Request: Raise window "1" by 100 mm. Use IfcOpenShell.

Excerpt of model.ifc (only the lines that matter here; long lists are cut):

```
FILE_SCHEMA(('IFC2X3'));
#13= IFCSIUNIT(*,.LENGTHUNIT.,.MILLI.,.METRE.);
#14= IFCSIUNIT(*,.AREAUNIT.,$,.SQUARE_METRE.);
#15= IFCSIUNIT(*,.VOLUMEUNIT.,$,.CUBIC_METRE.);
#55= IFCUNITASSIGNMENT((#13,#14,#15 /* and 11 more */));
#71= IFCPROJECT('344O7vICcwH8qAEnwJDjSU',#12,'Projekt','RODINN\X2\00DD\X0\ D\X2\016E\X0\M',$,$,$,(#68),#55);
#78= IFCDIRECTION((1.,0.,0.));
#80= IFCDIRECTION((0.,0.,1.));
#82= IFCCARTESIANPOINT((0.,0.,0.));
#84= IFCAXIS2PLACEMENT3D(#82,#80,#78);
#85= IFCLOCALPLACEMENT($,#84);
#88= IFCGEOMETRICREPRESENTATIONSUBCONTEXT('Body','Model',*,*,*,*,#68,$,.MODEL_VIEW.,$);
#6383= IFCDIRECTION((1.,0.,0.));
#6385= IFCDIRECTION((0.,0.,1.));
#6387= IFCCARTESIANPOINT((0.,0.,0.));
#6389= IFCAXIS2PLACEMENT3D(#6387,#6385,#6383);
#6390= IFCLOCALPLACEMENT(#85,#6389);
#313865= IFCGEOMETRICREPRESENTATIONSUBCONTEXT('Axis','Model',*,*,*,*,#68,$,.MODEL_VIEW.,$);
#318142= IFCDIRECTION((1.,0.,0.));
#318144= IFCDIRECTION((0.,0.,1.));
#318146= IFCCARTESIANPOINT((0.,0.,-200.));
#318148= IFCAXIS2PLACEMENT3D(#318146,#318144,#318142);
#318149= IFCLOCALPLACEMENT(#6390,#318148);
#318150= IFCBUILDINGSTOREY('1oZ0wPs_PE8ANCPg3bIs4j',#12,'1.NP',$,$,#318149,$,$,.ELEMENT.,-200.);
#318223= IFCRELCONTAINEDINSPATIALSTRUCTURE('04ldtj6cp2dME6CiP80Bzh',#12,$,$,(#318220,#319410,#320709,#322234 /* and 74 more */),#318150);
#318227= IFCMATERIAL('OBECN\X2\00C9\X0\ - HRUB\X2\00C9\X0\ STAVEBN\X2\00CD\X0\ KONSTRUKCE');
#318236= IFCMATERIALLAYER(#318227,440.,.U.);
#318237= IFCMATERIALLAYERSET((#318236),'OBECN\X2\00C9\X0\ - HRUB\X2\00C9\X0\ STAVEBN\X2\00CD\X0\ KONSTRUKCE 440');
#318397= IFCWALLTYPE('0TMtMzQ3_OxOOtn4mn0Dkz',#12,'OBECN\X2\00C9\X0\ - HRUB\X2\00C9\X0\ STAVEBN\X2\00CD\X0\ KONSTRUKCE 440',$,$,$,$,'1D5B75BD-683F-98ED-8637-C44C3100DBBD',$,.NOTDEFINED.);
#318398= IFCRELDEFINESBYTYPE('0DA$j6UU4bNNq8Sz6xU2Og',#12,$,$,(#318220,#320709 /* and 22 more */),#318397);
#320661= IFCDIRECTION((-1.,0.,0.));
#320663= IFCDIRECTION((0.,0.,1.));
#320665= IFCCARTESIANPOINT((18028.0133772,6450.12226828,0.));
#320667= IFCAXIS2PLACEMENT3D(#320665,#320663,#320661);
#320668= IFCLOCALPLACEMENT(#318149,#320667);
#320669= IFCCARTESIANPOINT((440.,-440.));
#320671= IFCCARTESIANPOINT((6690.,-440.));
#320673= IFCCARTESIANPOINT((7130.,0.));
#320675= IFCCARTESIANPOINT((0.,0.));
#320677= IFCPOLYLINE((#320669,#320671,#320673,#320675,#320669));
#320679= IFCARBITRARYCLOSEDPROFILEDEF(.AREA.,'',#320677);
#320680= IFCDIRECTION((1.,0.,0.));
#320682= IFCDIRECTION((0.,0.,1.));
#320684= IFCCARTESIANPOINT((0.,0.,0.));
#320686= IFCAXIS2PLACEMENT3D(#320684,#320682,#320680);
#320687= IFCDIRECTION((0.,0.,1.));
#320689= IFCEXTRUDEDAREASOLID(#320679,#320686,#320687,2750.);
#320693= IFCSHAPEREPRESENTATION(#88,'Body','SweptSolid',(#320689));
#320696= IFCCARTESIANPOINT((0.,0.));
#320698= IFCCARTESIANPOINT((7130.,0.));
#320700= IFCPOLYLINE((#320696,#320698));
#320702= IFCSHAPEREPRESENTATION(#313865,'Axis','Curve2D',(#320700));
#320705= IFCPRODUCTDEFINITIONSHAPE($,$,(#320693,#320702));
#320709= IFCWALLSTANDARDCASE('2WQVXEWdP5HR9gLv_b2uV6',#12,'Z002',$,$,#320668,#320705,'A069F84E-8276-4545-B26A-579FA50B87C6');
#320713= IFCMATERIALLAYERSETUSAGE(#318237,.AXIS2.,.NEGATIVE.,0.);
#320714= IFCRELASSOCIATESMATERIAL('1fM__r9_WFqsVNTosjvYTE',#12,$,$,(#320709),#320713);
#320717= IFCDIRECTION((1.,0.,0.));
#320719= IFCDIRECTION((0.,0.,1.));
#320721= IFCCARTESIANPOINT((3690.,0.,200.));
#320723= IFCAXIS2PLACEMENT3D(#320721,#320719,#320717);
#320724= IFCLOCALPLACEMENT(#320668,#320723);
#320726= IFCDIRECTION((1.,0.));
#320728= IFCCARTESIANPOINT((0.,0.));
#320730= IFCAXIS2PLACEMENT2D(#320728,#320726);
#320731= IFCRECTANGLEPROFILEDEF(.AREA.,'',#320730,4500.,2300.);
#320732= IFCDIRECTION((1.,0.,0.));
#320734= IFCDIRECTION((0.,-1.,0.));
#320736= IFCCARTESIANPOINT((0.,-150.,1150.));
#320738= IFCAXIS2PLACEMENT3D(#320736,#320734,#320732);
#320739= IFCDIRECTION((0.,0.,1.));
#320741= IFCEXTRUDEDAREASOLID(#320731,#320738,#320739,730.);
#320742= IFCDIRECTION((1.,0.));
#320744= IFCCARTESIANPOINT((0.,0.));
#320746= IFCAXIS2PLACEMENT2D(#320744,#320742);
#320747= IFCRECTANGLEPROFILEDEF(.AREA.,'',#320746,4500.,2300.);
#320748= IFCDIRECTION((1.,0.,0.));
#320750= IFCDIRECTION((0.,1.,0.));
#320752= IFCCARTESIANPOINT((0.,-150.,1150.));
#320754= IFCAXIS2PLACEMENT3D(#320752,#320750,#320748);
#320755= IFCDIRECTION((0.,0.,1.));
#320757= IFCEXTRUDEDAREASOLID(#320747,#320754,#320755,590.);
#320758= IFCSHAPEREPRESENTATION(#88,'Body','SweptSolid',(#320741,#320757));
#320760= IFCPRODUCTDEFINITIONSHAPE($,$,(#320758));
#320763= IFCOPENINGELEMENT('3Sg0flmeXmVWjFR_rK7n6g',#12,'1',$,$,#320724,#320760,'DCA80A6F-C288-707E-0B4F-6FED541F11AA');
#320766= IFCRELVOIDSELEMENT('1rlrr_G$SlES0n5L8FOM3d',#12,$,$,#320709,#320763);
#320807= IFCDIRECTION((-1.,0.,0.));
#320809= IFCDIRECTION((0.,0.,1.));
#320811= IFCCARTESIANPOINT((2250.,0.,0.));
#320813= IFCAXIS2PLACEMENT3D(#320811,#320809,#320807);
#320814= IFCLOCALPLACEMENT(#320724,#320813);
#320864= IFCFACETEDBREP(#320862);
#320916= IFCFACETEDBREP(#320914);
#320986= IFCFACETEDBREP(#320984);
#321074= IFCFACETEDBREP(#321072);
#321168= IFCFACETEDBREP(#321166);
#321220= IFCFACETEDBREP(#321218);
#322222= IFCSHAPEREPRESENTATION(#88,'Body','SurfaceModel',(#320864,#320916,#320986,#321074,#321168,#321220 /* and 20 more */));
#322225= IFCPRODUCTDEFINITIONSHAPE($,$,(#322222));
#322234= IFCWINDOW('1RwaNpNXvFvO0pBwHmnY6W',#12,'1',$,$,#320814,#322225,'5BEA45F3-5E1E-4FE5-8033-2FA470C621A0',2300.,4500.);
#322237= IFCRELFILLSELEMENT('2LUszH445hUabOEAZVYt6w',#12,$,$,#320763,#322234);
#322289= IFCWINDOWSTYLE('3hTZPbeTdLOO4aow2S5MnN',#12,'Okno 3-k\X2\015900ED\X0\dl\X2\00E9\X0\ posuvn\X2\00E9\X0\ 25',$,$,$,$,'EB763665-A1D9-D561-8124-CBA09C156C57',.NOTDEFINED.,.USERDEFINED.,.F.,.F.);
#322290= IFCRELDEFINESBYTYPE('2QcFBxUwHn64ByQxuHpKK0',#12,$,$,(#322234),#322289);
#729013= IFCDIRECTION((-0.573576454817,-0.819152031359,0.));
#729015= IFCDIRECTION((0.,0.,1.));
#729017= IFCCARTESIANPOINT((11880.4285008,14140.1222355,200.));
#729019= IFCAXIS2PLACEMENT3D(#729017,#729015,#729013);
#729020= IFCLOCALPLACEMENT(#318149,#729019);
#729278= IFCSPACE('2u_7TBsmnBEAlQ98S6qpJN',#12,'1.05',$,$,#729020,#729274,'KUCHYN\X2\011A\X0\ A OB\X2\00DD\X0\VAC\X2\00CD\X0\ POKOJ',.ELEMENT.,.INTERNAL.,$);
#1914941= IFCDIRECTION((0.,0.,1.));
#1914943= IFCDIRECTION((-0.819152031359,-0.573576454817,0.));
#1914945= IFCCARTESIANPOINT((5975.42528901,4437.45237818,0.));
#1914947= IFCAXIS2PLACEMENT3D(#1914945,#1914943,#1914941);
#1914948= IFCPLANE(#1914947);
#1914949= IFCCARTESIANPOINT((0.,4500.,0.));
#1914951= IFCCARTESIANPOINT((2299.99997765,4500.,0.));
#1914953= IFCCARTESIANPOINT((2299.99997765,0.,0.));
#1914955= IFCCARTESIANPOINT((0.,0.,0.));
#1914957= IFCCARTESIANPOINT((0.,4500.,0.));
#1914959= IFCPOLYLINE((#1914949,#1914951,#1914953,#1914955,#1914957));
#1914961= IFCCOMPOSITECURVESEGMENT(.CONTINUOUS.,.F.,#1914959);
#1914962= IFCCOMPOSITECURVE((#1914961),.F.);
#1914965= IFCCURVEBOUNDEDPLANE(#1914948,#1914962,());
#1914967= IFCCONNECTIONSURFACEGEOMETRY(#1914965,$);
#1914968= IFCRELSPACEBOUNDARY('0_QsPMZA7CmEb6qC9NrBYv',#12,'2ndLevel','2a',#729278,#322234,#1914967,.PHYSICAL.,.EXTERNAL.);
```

```python
import numpy as np
import ifcopenshell
import ifcopenshell.api.geometry
import ifcopenshell.util.placement
import ifcopenshell.util.unit

model = ifcopenshell.open("model.ifc")
unit_scale = ifcopenshell.util.unit.calculate_unit_scale(model)

window = model.by_guid("1RwaNpNXvFvO0pBwHmnY6W")
opening = window.FillsVoids[0].RelatingOpeningElement
dz = 0.1 / unit_scale

shift = np.array([0.0, 0.0, dz])
# The window is placed relative to its opening, so it follows when the opening moves.
matrix = ifcopenshell.util.placement.get_local_placement(opening.ObjectPlacement)
matrix[:3, 3] += shift
ifcopenshell.api.geometry.edit_object_placement(
    model, product=opening, matrix=matrix, is_si=False, should_transform_children=True
)

# Space boundary surfaces are stored in each space's coordinates; move them too.
for rel in window.ProvidesBoundaries:
    if not rel.ConnectionGeometry:
        continue
    surface = rel.ConnectionGeometry.SurfaceOnRelatingElement.BasisSurface
    space_matrix = ifcopenshell.util.placement.get_local_placement(rel.RelatingSpace.ObjectPlacement)
    point = np.array(surface.Position.Location.Coordinates) + space_matrix[:3, :3].T @ shift
    surface.Position = model.createIfcAxis2Placement3D(
        model.createIfcCartesianPoint(point.tolist()), surface.Position.Axis, surface.Position.RefDirection
    )

print(f"moved by {dz * unit_scale:+.3f} m")

model.write("model_v2.ifc")
```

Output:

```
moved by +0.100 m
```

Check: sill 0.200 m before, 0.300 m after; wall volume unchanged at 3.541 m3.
